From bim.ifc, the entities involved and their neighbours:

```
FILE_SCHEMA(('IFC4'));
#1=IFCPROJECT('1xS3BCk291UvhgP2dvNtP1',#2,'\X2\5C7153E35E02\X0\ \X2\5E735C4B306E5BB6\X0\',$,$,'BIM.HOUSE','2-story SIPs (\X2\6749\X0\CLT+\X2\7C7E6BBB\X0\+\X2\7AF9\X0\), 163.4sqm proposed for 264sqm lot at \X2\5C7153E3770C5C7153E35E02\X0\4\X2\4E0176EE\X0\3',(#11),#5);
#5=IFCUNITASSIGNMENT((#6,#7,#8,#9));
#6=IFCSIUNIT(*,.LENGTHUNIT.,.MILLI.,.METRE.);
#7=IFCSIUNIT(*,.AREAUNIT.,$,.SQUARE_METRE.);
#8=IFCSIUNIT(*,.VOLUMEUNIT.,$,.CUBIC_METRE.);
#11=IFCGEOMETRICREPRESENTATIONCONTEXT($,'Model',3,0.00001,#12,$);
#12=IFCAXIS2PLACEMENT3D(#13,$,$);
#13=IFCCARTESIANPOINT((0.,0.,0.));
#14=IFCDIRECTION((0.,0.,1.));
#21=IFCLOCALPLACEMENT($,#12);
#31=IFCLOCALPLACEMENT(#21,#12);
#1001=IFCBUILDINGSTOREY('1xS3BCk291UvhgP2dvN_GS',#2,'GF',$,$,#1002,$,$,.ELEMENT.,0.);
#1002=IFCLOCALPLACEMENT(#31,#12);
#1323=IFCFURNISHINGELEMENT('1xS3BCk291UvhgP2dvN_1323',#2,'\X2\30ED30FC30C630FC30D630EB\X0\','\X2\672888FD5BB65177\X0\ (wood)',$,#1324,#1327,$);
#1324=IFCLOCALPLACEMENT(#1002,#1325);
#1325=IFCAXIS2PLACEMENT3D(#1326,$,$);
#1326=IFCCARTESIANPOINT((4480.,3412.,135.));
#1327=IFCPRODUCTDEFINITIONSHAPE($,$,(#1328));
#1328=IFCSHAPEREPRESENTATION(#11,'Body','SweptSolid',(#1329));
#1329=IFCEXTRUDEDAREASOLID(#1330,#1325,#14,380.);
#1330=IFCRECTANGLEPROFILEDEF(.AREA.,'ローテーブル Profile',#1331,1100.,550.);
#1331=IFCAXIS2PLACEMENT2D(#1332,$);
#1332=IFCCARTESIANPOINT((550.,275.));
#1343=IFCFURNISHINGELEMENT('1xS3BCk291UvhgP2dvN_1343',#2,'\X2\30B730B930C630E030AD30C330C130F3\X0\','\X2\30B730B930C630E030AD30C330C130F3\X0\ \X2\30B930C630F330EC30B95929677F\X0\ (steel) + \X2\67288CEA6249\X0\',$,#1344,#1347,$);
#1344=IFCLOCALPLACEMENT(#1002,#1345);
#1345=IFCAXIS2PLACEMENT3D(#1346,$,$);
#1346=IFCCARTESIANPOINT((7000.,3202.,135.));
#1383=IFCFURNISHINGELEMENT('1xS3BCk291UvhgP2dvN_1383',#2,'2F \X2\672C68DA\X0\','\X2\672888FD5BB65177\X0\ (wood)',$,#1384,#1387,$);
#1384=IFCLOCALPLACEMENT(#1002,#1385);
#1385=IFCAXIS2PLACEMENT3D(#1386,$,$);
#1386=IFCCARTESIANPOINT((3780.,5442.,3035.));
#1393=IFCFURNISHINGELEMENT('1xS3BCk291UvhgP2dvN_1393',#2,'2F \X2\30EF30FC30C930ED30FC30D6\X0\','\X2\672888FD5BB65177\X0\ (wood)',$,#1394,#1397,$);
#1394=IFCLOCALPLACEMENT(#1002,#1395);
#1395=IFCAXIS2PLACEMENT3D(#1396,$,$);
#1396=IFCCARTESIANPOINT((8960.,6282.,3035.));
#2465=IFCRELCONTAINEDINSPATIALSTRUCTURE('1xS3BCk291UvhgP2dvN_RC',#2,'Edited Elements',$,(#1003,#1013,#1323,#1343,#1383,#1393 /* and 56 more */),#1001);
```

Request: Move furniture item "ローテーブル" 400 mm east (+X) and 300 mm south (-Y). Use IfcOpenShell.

```python
import ifcopenshell
import ifcopenshell.api.geometry
import ifcopenshell.util.placement
import ifcopenshell.util.unit

model = ifcopenshell.open("bim.ifc")
unit_scale = ifcopenshell.util.unit.calculate_unit_scale(model)

item = model.by_guid("1xS3BCk291UvhgP2dvN_1323")
matrix = ifcopenshell.util.placement.get_local_placement(item.ObjectPlacement)
matrix[0, 3] += 0.4 / unit_scale
matrix[1, 3] -= 0.3 / unit_scale
ifcopenshell.api.geometry.edit_object_placement(model, product=item, matrix=matrix, is_si=False)

print(ifcopenshell.util.placement.get_local_placement(item.ObjectPlacement).round(3) + 0.0)

model.write("bim_rev.ifc")
```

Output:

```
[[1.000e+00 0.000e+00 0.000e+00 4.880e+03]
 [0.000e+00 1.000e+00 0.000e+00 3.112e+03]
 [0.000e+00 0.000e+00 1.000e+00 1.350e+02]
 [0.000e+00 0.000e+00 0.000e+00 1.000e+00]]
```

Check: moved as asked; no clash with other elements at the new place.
